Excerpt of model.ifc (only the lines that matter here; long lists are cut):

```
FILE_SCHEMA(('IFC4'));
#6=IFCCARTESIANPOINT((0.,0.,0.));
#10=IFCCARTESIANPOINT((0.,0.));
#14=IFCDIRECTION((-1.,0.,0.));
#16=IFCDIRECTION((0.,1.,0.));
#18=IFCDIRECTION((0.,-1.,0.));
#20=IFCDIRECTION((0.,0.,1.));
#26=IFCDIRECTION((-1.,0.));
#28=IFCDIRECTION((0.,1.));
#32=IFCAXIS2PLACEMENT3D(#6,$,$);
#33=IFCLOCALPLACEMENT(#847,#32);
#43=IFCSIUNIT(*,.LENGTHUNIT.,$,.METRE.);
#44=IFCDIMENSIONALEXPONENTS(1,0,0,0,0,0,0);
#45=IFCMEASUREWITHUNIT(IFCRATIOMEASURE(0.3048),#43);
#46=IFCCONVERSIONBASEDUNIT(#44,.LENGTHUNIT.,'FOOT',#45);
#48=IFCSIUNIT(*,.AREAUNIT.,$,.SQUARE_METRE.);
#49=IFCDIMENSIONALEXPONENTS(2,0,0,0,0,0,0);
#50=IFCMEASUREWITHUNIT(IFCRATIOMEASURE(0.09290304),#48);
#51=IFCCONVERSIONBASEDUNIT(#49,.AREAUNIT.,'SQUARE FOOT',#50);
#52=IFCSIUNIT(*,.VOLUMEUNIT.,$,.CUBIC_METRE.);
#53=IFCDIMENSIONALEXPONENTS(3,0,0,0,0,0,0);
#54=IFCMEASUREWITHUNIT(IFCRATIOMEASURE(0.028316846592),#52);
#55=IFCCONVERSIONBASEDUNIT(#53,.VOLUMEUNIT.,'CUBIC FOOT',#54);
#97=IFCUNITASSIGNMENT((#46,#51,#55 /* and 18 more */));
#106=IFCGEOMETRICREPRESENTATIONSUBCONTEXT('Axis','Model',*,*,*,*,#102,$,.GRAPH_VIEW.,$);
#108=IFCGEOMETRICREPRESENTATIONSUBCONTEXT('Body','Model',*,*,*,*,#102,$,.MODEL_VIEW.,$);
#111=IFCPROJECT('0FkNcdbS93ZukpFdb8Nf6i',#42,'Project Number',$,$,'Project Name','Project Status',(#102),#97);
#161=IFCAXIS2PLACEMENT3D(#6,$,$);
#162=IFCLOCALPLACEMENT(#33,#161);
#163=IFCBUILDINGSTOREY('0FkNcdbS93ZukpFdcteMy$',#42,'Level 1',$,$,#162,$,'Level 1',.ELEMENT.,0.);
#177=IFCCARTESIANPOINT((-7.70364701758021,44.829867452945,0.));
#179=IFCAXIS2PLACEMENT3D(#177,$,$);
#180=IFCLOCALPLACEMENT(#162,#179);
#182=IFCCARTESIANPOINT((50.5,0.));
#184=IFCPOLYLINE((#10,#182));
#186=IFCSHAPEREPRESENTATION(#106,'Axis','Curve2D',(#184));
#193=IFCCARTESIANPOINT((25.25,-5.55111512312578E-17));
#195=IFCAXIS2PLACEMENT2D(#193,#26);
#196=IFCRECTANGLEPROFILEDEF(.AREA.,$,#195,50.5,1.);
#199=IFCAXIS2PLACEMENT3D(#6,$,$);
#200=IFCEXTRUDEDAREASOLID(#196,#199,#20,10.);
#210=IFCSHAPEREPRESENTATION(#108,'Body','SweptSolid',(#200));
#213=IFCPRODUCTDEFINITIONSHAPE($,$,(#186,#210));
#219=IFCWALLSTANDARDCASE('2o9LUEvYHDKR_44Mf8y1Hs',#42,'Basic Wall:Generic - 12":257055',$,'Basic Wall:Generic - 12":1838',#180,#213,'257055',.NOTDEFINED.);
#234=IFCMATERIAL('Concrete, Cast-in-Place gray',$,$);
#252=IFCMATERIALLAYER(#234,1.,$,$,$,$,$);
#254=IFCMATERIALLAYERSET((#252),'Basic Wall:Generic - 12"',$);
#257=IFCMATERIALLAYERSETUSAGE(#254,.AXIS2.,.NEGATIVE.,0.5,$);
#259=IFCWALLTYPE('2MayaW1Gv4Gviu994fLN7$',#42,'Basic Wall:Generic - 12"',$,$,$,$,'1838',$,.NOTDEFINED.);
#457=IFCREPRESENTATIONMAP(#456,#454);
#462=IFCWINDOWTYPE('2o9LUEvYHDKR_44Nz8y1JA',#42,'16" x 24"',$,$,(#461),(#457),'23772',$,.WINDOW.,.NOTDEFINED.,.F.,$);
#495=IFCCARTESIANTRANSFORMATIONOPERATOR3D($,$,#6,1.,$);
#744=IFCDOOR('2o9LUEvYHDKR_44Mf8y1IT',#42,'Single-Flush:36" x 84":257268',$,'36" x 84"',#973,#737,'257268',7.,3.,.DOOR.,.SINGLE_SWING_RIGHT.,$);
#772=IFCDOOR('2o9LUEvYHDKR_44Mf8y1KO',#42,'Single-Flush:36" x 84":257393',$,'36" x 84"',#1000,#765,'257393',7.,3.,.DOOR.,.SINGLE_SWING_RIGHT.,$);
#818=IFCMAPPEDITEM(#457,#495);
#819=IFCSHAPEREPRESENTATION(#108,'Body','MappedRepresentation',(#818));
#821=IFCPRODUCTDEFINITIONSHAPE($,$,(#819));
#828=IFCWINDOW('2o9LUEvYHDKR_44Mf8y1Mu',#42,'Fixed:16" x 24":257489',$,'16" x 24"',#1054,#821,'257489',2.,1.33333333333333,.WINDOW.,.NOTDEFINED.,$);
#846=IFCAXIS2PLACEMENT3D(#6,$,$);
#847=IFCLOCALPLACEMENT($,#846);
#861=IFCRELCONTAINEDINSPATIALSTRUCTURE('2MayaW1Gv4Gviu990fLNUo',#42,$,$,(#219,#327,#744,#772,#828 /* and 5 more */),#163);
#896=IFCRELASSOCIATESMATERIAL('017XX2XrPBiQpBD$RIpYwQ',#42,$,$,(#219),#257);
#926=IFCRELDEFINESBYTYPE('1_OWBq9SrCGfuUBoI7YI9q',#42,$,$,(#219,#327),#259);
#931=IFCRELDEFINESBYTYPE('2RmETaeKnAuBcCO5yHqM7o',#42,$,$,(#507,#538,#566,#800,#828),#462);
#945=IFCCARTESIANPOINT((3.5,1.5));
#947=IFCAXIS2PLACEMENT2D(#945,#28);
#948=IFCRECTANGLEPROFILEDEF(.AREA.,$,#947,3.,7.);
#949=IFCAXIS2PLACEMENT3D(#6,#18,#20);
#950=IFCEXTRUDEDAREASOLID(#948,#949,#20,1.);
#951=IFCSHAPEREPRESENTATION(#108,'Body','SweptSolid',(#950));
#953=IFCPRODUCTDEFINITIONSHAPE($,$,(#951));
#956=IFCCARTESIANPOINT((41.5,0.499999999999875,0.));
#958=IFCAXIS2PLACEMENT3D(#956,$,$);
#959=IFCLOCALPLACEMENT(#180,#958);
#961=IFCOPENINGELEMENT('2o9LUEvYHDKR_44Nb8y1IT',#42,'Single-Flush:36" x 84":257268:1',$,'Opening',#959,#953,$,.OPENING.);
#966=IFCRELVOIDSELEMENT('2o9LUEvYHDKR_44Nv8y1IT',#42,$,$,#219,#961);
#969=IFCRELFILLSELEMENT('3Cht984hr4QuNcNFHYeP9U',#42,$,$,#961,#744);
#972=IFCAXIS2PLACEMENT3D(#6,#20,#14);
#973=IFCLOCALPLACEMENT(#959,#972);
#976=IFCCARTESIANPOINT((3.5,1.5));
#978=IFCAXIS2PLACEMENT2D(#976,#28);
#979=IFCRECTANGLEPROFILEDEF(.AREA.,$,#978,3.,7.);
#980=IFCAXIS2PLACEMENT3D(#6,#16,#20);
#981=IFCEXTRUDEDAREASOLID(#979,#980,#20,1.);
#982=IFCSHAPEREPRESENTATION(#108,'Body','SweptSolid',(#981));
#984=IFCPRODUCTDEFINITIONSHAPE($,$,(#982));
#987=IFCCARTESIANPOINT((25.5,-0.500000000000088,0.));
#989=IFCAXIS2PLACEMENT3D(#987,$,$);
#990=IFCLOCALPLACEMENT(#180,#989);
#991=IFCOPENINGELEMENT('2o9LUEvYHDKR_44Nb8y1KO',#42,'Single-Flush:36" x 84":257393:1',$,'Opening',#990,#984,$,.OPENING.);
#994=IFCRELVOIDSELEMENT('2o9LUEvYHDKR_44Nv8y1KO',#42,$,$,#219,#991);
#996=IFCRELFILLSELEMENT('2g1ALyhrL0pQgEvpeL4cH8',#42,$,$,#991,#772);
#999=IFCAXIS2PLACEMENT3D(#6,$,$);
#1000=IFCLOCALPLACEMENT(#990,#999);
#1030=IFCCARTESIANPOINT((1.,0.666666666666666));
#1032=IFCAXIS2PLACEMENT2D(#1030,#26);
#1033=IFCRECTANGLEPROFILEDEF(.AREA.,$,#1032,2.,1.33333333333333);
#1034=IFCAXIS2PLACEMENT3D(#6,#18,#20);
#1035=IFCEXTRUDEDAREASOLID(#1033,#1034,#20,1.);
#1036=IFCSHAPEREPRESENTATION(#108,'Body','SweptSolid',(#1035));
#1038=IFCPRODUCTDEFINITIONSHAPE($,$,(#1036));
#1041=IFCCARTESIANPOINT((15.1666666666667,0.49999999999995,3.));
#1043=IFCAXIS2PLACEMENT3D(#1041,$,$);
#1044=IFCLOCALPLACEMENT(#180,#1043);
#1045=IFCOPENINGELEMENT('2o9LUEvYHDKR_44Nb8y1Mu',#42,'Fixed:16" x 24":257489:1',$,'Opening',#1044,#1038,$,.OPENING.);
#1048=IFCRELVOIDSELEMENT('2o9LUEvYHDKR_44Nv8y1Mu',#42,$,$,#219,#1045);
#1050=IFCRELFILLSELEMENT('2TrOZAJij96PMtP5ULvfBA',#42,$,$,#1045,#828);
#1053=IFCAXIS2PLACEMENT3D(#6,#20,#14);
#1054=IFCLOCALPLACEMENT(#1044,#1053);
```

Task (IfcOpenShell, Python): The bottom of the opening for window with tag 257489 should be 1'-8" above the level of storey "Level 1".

```python
import numpy as np
import ifcopenshell
import ifcopenshell.api.geometry
import ifcopenshell.geom
import ifcopenshell.util.element
import ifcopenshell.util.placement
import ifcopenshell.util.shape
import ifcopenshell.util.unit

model = ifcopenshell.open("model.ifc")
unit_scale = ifcopenshell.util.unit.calculate_unit_scale(model)

window = model.by_id(828)
opening = window.FillsVoids[0].RelatingOpeningElement
storey = ifcopenshell.util.element.get_container(window, ifc_class="IfcBuildingStorey")
level = ifcopenshell.util.placement.get_local_placement(storey.ObjectPlacement)[2, 3]

# The opening's origin need not be at the sill, so measure its lowest point.
shape = ifcopenshell.geom.create_shape(ifcopenshell.geom.settings(), opening)
bottom = ifcopenshell.util.shape.get_shape_bottom_elevation(shape, shape.geometry) / unit_scale
dz = level + 20 * 0.0254 / unit_scale - bottom

shift = np.array([0.0, 0.0, dz])
# The window is placed relative to its opening, so it follows when the opening moves.
matrix = ifcopenshell.util.placement.get_local_placement(opening.ObjectPlacement)
matrix[:3, 3] += shift
ifcopenshell.api.geometry.edit_object_placement(
    model, product=opening, matrix=matrix, is_si=False, should_transform_children=True
)

print(f"moved by {dz * unit_scale:+.3f} m")

model.write("model_rev.ifc")
```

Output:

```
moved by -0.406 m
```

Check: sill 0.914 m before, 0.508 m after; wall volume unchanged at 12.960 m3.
